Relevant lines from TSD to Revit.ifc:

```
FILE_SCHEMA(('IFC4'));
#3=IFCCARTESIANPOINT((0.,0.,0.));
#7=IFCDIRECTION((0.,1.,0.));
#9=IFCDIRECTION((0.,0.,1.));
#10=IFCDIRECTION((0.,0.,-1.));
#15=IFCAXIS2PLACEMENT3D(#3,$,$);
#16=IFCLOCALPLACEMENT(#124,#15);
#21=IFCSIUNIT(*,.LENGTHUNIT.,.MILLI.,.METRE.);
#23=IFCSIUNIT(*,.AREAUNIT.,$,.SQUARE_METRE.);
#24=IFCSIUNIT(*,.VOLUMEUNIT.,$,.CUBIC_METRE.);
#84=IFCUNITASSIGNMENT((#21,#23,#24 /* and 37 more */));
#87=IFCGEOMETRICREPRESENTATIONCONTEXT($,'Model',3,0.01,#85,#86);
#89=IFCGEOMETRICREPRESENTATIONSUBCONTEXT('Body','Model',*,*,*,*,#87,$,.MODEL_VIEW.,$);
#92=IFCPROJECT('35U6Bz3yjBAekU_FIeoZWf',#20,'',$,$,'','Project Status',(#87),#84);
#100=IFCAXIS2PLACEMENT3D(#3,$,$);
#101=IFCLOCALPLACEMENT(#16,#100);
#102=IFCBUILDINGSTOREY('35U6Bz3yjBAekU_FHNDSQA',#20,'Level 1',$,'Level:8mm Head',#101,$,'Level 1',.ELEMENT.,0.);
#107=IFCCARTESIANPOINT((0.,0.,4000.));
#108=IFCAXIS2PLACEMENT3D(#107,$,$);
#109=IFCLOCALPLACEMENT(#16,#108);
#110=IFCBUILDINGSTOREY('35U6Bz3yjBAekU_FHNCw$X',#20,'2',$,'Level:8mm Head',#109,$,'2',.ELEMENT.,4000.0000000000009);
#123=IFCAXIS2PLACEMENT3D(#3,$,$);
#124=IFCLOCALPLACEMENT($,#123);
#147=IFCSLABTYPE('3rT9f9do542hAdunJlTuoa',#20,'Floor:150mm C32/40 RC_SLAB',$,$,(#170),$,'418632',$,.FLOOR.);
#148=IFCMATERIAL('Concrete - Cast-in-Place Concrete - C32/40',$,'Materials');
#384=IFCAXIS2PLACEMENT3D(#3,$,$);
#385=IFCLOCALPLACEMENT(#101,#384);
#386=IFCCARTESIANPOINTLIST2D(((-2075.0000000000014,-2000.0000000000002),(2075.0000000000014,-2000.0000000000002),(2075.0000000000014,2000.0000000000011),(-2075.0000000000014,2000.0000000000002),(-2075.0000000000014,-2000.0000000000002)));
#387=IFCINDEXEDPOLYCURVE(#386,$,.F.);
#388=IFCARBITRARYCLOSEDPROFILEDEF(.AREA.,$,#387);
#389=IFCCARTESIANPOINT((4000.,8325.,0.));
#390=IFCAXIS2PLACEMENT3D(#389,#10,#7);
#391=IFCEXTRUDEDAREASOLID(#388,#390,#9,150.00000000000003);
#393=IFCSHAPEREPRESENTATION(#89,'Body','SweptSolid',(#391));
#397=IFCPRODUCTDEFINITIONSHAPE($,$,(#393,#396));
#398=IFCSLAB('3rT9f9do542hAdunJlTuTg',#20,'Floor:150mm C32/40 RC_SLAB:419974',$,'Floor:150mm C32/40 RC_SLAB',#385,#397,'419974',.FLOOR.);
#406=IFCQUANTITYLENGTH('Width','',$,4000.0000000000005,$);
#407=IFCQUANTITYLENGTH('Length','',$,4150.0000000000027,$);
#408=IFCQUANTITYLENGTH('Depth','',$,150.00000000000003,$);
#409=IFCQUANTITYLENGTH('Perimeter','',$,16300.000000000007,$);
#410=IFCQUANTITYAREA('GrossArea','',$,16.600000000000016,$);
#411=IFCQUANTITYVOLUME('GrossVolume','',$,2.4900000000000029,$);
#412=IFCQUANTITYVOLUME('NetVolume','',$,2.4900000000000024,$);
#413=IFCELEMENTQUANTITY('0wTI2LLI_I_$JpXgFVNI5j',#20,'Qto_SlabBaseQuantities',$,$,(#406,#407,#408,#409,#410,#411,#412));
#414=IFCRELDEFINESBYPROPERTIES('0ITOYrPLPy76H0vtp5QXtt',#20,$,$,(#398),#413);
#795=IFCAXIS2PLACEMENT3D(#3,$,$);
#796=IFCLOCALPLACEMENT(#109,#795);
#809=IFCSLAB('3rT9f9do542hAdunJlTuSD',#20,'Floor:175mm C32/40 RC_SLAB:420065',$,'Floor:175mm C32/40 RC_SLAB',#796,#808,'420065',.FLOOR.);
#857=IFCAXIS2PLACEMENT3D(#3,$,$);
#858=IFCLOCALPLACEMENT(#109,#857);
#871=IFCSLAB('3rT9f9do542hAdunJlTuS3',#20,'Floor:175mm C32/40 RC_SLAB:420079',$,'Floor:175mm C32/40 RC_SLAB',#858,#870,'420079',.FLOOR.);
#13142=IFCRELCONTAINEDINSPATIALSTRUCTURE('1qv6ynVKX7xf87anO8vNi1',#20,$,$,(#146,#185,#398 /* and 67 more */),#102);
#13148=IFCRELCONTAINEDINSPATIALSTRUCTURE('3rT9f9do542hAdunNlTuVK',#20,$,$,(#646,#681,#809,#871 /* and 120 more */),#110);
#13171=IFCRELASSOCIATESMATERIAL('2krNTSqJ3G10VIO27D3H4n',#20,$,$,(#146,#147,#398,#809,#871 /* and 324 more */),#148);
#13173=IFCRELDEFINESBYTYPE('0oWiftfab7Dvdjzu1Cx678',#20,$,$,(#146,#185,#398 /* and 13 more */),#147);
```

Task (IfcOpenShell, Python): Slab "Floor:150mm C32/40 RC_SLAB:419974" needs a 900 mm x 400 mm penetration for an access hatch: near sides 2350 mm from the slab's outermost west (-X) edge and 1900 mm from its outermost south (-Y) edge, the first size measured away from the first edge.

```python
import numpy as np
import ifcopenshell
import ifcopenshell.api.feature
import ifcopenshell.api.geometry
import ifcopenshell.api.pset
import ifcopenshell.api.root
import ifcopenshell.geom
import ifcopenshell.util.element
import ifcopenshell.util.placement
import ifcopenshell.util.representation
import ifcopenshell.util.shape
import ifcopenshell.util.unit

model = ifcopenshell.open("TSD to Revit.ifc")
unit_scale = ifcopenshell.util.unit.calculate_unit_scale(model)
volume_scale = ifcopenshell.util.unit.calculate_unit_scale(model, "VOLUMEUNIT")
settings = ifcopenshell.geom.settings()


def volume(element):
    """Net volume in cubic metres, openings subtracted."""
    shape = ifcopenshell.geom.create_shape(settings, element)
    return ifcopenshell.util.shape.get_volume(shape.geometry)


slab = model.by_guid("3rT9f9do542hAdunJlTuTg")
before = volume(slab)

# Extent in the slab's own axes, in metres. The edges named are its -X and -Y sides.
slab_shape = ifcopenshell.geom.create_shape(settings, slab)
vertices = ifcopenshell.util.shape.get_vertices(slab_shape.geometry)
x_min, y_min, bottom = vertices.min(axis=0)
top = vertices[:, 2].max()

opening = ifcopenshell.api.root.create_entity(model, ifc_class="IfcOpeningElement", name="Access hatch opening", predefined_type="OPENING")
context = ifcopenshell.util.representation.get_context(model, "Model", "Body", "MODEL_VIEW")
width, depth = 0.9, 0.4
outline = [(0.0, 0.0), (width, 0.0), (width, depth), (0.0, depth), (0.0, 0.0)]
# Overshoot both faces by 50 mm so the cut is clean.
shape = ifcopenshell.api.geometry.add_slab_representation(
    model, context=context, depth=top - bottom + 0.1, polyline=outline
)
ifcopenshell.api.geometry.assign_representation(model, product=opening, representation=shape)

matrix = ifcopenshell.util.placement.get_local_placement(slab.ObjectPlacement)
matrix[:, 3] = matrix @ np.append(np.array([x_min + 2.35, y_min + 1.9, bottom - 0.05]) / unit_scale, 1.0)
ifcopenshell.api.geometry.edit_object_placement(model, product=opening, matrix=matrix, is_si=False)
ifcopenshell.api.feature.add_feature(model, feature=opening, element=slab)

after = volume(slab)

# Update the slab's stored quantities.
qto = model.by_id(ifcopenshell.util.element.get_pset(slab, "Qto_SlabBaseQuantities", should_inherit=False)["id"])
ifcopenshell.api.pset.edit_qto(model, qto=qto, properties={"NetVolume": after / volume_scale})

print(f"slab volume {before:.3f} -> {after:.3f} m3")

model.write("TSD to Revit_edited.ifc")
```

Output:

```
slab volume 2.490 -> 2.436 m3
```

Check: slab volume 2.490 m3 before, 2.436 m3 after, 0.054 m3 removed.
